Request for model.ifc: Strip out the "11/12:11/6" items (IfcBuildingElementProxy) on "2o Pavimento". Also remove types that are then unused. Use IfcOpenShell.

First a look at what the model holds.

```python
import ifcopenshell
import ifcopenshell.util.element

model = ifcopenshell.open("model.ifc")
print(model.schema)
storey = next(s for s in model.by_type("IfcBuildingStorey") if s.Name == "2o Pavimento")
proxies = [e for e in ifcopenshell.util.element.get_decomposition(storey) if e.is_a("IfcBuildingElementProxy")]
seen = {}
for e in proxies:
    element_type = ifcopenshell.util.element.get_type(e)
    name = element_type.Name if element_type not in (None, e) else None
    seen[name] = seen.get(name, 0) + 1
for name, count in sorted(seen.items(), key=str):
    print(count, "x", name)
```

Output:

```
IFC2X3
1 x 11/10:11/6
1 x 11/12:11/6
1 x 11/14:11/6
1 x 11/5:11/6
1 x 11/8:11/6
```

```python
import ifcopenshell
import ifcopenshell.api.root
import ifcopenshell.util.element

model = ifcopenshell.open("model.ifc")

storey = next(s for s in model.by_type("IfcBuildingStorey") if s.Name == "2o Pavimento")
proxies = [e for e in ifcopenshell.util.element.get_decomposition(storey) if e.is_a("IfcBuildingElementProxy")]
targets = [e for e in proxies if (t := ifcopenshell.util.element.get_type(e)) not in (None, e) and t.Name == "11/12:11/6"]
types = {ifcopenshell.util.element.get_type(e) for e in targets} - {None, *targets}

for e in targets:
    ifcopenshell.api.root.remove_product(model, product=e)
print(len(targets), "removed")

unused = [t for t in types if not ifcopenshell.util.element.get_types(t)]
for t in unused:
    ifcopenshell.api.root.remove_product(model, product=t)
print(len(unused), "unused types removed")

model.write("model_rev.ifc")
```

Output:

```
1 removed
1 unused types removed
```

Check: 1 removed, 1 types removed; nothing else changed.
